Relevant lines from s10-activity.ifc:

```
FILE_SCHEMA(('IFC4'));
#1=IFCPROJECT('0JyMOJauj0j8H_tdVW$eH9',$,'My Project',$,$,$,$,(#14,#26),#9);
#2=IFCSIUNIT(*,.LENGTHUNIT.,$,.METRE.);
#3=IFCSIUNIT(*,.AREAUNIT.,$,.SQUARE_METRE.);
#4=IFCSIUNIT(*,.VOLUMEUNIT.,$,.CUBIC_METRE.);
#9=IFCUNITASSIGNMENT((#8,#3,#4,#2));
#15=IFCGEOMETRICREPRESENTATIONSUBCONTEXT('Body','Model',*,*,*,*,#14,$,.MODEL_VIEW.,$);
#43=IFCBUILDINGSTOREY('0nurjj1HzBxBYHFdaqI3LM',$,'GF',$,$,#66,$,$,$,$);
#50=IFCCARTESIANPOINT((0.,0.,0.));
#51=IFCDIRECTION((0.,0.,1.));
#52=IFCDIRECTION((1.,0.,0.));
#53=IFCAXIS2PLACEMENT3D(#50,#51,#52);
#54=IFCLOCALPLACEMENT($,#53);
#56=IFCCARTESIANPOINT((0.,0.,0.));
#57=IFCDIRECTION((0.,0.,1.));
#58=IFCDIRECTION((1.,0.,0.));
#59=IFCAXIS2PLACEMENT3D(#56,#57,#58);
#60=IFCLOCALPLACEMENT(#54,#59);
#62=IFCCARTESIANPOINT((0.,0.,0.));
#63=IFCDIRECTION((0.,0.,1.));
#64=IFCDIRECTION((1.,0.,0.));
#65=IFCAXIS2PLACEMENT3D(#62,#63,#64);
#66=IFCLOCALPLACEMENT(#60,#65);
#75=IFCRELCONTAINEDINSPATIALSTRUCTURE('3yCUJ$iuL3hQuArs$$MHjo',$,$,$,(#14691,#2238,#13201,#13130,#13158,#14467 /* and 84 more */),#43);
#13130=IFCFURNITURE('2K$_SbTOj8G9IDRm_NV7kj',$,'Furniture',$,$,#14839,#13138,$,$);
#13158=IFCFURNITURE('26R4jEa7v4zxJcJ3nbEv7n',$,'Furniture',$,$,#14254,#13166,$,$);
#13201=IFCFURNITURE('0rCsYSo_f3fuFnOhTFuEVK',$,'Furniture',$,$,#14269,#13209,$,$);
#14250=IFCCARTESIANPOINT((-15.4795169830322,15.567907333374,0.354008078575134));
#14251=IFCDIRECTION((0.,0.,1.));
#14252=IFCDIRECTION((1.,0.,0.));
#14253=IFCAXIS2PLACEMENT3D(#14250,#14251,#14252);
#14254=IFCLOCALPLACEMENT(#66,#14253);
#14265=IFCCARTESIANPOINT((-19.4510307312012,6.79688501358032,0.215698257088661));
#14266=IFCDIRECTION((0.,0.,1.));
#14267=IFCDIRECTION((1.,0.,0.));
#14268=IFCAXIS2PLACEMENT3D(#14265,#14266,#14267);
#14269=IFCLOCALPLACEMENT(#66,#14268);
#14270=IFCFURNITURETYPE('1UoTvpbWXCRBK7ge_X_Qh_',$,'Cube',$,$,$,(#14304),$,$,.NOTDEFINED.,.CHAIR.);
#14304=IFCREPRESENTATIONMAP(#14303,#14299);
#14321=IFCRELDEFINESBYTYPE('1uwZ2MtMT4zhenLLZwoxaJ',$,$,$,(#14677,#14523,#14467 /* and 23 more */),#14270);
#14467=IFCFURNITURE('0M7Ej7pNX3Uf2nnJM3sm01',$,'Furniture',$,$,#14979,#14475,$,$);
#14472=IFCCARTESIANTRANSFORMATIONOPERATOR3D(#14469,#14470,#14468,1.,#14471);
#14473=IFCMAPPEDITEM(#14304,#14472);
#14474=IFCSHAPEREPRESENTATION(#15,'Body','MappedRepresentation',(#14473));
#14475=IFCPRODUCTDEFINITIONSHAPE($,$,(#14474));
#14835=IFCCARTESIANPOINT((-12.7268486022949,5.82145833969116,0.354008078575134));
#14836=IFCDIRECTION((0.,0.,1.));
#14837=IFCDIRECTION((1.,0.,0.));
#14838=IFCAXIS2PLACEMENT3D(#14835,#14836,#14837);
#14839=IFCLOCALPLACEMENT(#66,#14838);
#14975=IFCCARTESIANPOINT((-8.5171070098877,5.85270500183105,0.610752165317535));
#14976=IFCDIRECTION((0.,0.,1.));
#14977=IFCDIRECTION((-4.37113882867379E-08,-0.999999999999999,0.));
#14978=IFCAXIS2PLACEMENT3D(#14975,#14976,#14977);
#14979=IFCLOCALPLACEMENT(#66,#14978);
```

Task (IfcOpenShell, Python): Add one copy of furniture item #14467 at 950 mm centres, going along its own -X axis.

```python
import ifcopenshell
import ifcopenshell.api.geometry
import ifcopenshell.api.root
import ifcopenshell.util.element
import ifcopenshell.util.placement

model = ifcopenshell.open("s10-activity.ifc")

source = model.by_guid("0M7Ej7pNX3Uf2nnJM3sm01")
base = ifcopenshell.util.placement.get_local_placement(source.ObjectPlacement)
step = -base[:3, 0] * 0.95

for i in range(1, 2):
    copy = ifcopenshell.api.root.copy_class(model, product=source)
    copy.Representation = ifcopenshell.util.element.copy_deep(
        model, source.Representation, exclude=["IfcGeometricRepresentationContext", "IfcRepresentationMap"]
    )
    matrix = base.copy()
    matrix[:3, 3] += i * step
    print("added at", matrix[:3, 3].round(3) + 0.0)
    ifcopenshell.api.geometry.edit_object_placement(model, product=copy, matrix=matrix, is_si=False)

model.write("s10-activity_updated.ifc")
```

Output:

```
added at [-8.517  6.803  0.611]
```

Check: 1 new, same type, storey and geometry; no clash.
